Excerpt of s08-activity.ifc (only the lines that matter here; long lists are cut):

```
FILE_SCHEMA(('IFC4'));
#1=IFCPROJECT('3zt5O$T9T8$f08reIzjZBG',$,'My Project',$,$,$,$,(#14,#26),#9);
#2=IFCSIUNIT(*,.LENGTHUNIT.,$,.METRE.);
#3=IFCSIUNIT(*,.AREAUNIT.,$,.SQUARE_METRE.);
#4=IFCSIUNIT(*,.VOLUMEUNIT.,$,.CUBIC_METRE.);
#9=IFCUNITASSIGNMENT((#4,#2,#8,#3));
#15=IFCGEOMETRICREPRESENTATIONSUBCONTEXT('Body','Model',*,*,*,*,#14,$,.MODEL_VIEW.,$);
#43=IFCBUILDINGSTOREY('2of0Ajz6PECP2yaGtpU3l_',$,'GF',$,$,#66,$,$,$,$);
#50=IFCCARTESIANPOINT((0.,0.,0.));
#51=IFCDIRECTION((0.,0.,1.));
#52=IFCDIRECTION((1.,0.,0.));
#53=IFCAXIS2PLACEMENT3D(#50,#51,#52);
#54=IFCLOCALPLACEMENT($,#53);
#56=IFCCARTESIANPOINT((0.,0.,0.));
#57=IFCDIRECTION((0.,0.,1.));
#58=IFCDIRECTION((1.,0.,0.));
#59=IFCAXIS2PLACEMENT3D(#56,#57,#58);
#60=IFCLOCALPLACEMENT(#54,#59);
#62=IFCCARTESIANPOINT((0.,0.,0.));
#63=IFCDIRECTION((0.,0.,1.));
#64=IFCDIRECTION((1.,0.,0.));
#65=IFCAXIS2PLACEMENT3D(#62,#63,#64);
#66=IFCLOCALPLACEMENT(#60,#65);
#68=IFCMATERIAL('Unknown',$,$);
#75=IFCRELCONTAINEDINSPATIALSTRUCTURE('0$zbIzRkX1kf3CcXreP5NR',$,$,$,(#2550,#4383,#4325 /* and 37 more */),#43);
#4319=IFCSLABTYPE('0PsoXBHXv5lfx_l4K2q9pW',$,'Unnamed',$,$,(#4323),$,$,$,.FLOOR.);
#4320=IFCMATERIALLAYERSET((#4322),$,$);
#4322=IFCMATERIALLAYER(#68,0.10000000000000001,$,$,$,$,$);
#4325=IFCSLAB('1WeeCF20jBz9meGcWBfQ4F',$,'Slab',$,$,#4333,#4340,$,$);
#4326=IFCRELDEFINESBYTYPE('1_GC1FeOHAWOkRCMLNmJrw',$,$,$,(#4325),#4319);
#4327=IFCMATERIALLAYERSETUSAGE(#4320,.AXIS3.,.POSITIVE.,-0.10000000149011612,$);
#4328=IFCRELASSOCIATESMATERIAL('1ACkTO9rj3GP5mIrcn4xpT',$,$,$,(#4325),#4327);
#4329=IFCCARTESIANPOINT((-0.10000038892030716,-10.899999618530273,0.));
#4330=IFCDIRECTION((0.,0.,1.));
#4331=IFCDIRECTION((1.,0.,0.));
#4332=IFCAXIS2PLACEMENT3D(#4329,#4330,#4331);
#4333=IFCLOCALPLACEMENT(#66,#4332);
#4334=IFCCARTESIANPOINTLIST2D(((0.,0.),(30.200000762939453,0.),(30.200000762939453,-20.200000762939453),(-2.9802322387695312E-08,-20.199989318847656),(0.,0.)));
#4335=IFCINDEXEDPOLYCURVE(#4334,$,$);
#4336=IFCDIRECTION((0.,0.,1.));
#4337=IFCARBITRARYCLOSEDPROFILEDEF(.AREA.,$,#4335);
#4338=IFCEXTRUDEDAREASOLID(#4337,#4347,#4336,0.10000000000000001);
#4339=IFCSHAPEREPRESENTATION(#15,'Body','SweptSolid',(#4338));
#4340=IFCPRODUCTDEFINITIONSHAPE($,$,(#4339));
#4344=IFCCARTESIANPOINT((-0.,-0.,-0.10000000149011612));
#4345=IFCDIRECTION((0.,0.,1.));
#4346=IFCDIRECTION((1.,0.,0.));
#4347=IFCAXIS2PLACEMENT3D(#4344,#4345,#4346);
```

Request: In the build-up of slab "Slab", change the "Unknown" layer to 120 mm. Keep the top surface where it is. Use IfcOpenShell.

```python
import ifcopenshell
import ifcopenshell.util.element
import ifcopenshell.util.representation

model = ifcopenshell.open("s08-activity.ifc")

layer_set = model.by_id(4320)
layer = next(l for l in layer_set.MaterialLayers if l.Material and l.Material.Name == "Unknown")
change = 0.12 - layer.LayerThickness
layer.LayerThickness += change

# Geometry does not follow the layer set by itself.
slabs = [e for e in ifcopenshell.util.element.get_elements_by_material(model, layer_set) if e.is_a("IfcSlab")]
for slab in sorted(slabs, key=lambda e: e.id()):
    body = ifcopenshell.util.representation.get_representation(slab, "Model", "Body")
    solid = body.Items[0]
    old_depth = solid.Depth
    solid.Depth += change
    # Extruded upwards: lower the start of the extrusion so the top stays.
    x, y, z = solid.Position.Location.Coordinates
    solid.Position.Location = model.createIfcCartesianPoint((x, y, z - change))
    print(slab.id(), f"{old_depth:g} -> {solid.Depth:g}")

# The layers are counted up from the underside, which has moved.
for usage in {ifcopenshell.util.element.get_material(slab) for slab in slabs}:
    usage.OffsetFromReferenceLine -= change

model.write("s08-activity_updated.ifc")
```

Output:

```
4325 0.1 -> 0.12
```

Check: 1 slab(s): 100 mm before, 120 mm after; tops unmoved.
